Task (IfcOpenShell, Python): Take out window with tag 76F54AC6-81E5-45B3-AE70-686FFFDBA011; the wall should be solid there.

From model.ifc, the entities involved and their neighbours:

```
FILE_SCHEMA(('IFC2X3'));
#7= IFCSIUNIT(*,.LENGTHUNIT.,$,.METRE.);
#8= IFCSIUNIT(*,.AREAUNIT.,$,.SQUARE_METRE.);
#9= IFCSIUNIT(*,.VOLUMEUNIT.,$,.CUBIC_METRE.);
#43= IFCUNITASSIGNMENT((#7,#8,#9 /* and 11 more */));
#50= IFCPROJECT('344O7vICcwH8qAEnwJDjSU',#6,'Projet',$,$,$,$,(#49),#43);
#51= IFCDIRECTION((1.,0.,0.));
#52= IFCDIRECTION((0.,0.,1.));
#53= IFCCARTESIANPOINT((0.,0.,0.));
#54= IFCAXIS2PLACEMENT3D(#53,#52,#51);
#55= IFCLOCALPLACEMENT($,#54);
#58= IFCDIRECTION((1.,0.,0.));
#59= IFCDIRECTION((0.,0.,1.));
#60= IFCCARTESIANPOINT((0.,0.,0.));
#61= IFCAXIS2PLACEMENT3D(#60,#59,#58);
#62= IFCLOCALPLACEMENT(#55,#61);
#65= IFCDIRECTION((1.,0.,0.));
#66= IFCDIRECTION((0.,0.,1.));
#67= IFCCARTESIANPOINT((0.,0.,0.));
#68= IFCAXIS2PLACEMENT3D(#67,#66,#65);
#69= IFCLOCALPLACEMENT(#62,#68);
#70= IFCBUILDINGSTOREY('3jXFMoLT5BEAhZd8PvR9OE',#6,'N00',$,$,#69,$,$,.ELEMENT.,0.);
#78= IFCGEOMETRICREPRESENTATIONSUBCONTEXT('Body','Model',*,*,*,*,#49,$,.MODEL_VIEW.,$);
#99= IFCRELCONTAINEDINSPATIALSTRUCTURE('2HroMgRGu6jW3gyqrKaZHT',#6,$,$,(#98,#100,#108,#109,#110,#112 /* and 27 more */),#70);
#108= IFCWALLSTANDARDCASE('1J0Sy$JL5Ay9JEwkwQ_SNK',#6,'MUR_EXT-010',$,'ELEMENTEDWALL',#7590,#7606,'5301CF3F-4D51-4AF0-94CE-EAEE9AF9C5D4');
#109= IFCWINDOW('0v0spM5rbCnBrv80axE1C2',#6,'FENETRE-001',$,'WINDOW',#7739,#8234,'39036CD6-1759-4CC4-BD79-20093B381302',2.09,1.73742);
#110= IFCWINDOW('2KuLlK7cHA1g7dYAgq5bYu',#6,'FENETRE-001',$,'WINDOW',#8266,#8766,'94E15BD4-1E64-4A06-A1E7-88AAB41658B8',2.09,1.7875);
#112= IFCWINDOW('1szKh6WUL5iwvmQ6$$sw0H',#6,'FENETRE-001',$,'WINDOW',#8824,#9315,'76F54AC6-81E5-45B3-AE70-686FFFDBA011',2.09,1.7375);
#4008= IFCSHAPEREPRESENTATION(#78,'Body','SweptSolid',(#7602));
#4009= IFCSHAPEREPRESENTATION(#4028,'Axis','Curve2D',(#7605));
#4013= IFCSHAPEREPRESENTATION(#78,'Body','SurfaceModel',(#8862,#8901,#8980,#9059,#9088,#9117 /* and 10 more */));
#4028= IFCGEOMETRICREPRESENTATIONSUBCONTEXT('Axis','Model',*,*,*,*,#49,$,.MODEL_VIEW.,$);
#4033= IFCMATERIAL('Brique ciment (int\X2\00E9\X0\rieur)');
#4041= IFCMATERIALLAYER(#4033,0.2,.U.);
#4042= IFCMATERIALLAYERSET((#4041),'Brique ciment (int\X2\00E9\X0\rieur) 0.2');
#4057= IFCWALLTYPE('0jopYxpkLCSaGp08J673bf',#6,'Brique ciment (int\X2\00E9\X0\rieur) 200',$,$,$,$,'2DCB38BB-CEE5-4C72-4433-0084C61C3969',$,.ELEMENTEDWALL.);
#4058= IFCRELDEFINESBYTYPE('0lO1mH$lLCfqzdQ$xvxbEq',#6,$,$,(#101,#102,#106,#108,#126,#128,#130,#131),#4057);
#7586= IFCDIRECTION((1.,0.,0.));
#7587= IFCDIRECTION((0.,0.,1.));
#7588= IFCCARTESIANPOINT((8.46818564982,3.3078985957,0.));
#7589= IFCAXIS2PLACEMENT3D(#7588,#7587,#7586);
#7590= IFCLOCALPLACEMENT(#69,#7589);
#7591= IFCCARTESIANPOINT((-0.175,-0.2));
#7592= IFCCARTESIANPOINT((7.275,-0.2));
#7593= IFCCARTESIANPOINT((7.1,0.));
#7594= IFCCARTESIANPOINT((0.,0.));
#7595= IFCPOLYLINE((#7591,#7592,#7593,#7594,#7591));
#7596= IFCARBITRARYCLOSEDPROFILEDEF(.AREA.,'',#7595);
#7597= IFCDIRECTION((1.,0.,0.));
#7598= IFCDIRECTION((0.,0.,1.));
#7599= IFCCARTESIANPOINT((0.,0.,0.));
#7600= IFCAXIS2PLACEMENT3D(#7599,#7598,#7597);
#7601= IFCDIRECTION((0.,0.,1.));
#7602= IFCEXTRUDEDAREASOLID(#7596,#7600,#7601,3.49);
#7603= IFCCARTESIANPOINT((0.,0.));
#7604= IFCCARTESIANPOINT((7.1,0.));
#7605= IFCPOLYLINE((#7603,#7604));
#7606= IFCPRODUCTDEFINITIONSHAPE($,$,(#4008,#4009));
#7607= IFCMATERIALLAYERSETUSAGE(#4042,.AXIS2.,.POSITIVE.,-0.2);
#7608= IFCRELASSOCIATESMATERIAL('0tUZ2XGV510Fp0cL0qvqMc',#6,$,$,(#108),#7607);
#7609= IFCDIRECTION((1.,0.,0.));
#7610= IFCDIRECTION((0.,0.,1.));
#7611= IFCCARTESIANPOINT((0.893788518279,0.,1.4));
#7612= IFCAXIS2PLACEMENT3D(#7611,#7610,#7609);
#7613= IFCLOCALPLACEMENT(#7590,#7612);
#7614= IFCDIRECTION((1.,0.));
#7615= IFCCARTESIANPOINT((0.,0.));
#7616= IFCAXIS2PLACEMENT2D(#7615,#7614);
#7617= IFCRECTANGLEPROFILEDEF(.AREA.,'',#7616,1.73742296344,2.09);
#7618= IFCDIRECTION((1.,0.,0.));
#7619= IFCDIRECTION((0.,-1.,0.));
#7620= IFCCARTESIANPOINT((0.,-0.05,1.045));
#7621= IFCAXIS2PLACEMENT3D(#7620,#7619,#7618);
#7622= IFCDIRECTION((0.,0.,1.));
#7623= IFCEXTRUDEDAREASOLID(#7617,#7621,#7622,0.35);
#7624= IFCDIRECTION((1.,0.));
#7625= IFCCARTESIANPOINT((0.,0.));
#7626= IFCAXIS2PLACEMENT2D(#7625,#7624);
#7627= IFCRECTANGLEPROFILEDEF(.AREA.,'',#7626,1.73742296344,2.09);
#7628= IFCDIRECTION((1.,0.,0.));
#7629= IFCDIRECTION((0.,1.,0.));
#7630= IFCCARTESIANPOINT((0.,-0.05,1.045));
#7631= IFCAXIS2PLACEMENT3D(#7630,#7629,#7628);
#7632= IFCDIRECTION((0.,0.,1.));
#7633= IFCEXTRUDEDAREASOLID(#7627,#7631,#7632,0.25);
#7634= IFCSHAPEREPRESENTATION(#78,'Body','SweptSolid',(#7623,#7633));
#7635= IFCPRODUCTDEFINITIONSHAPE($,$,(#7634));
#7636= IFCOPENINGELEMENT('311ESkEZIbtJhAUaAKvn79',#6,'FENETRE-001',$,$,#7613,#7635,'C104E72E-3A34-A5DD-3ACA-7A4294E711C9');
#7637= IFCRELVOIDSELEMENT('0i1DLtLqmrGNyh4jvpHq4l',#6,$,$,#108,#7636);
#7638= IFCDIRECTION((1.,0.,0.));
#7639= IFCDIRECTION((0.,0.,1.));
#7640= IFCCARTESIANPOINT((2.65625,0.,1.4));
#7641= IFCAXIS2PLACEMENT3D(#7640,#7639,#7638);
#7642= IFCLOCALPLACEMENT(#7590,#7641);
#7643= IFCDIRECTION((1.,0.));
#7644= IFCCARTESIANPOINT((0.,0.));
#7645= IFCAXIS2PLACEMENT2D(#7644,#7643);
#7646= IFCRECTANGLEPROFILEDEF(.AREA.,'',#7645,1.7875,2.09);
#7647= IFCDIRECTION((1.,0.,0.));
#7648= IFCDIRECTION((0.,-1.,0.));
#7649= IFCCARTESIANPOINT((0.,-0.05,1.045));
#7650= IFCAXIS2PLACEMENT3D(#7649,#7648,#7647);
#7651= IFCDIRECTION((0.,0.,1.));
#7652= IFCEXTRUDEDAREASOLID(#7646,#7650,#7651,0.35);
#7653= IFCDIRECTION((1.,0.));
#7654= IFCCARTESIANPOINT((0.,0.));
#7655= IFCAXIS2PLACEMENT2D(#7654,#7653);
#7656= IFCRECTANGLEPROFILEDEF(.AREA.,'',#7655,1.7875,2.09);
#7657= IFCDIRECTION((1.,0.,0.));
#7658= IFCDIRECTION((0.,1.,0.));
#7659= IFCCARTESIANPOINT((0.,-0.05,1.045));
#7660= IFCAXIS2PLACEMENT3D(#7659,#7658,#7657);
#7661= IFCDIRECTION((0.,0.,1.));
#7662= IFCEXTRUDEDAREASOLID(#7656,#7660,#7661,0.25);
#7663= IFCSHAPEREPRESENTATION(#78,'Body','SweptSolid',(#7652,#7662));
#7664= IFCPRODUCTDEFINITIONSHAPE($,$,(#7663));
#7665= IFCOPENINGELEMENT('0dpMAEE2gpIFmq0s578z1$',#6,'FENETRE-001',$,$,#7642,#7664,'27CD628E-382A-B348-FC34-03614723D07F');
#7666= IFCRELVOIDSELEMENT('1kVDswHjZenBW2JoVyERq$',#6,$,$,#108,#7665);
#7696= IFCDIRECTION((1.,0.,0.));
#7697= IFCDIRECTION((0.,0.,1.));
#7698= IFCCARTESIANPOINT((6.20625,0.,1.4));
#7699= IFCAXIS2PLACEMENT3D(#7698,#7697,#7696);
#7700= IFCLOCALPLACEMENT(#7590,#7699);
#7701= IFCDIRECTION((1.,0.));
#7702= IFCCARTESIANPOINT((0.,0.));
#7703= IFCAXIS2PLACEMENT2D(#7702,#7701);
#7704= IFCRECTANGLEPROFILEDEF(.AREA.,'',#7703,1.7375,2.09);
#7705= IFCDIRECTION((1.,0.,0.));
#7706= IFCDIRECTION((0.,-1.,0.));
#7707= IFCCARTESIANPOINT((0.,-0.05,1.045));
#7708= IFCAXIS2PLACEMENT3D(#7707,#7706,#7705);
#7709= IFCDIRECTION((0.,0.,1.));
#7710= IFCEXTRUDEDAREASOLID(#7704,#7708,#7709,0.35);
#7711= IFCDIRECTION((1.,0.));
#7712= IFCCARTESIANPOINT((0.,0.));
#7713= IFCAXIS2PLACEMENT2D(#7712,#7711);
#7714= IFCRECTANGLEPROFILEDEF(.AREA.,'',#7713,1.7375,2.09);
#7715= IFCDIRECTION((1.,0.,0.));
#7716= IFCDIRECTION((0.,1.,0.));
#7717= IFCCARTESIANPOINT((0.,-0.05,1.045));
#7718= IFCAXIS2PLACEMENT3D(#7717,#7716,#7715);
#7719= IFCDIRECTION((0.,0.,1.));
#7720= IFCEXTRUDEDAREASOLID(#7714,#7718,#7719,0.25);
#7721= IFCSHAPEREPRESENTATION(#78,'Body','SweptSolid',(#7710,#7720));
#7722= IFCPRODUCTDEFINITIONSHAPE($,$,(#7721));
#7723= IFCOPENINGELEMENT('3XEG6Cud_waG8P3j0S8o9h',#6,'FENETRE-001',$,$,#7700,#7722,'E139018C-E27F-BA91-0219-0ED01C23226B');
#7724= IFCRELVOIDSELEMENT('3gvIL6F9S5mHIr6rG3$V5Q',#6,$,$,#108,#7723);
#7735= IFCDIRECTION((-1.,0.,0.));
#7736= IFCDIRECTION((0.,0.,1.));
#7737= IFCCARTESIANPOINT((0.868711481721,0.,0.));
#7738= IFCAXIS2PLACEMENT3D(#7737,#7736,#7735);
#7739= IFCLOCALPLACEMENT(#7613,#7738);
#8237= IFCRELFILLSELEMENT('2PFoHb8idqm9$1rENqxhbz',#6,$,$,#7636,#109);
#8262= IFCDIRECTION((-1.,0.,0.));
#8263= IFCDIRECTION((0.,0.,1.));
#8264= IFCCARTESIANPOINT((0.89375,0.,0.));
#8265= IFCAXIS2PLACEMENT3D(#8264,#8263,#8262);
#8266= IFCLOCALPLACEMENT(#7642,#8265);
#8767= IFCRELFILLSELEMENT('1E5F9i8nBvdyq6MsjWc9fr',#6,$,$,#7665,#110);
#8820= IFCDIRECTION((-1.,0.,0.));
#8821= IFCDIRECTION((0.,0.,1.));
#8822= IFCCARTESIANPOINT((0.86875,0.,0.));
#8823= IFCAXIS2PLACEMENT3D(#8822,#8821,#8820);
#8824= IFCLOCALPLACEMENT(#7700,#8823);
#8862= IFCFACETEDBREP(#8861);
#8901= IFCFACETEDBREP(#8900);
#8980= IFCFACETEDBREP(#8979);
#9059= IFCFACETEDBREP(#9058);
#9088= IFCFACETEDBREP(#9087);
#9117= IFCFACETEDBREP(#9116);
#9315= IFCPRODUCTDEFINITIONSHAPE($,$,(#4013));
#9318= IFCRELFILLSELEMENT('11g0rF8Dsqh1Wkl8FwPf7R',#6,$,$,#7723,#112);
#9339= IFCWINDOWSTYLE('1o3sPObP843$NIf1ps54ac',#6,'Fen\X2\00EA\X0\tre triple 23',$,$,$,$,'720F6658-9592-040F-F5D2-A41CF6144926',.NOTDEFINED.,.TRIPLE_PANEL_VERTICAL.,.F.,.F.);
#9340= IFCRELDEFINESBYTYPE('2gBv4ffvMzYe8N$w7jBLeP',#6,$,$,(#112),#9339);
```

```python
import ifcopenshell
import ifcopenshell.api.feature
import ifcopenshell.api.root
import ifcopenshell.geom
import ifcopenshell.util.shape

model = ifcopenshell.open("model.ifc")
settings = ifcopenshell.geom.settings()


def volume(element):
    """Net volume in cubic metres, openings subtracted."""
    shape = ifcopenshell.geom.create_shape(settings, element)
    return ifcopenshell.util.shape.get_volume(shape.geometry)


window = model.by_guid("1szKh6WUL5iwvmQ6$$sw0H")
opening = window.FillsVoids[0].RelatingOpeningElement
wall = opening.VoidsElements[0].RelatingBuildingElement
before = volume(wall)

ifcopenshell.api.root.remove_product(model, product=window)
ifcopenshell.api.feature.remove_feature(model, feature=opening)

after = volume(wall)

print(f"wall volume {before:.3f} -> {after:.3f} m3")

model.write("model_edited.ifc")
```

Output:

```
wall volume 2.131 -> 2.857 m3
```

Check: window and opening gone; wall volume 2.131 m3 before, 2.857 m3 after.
